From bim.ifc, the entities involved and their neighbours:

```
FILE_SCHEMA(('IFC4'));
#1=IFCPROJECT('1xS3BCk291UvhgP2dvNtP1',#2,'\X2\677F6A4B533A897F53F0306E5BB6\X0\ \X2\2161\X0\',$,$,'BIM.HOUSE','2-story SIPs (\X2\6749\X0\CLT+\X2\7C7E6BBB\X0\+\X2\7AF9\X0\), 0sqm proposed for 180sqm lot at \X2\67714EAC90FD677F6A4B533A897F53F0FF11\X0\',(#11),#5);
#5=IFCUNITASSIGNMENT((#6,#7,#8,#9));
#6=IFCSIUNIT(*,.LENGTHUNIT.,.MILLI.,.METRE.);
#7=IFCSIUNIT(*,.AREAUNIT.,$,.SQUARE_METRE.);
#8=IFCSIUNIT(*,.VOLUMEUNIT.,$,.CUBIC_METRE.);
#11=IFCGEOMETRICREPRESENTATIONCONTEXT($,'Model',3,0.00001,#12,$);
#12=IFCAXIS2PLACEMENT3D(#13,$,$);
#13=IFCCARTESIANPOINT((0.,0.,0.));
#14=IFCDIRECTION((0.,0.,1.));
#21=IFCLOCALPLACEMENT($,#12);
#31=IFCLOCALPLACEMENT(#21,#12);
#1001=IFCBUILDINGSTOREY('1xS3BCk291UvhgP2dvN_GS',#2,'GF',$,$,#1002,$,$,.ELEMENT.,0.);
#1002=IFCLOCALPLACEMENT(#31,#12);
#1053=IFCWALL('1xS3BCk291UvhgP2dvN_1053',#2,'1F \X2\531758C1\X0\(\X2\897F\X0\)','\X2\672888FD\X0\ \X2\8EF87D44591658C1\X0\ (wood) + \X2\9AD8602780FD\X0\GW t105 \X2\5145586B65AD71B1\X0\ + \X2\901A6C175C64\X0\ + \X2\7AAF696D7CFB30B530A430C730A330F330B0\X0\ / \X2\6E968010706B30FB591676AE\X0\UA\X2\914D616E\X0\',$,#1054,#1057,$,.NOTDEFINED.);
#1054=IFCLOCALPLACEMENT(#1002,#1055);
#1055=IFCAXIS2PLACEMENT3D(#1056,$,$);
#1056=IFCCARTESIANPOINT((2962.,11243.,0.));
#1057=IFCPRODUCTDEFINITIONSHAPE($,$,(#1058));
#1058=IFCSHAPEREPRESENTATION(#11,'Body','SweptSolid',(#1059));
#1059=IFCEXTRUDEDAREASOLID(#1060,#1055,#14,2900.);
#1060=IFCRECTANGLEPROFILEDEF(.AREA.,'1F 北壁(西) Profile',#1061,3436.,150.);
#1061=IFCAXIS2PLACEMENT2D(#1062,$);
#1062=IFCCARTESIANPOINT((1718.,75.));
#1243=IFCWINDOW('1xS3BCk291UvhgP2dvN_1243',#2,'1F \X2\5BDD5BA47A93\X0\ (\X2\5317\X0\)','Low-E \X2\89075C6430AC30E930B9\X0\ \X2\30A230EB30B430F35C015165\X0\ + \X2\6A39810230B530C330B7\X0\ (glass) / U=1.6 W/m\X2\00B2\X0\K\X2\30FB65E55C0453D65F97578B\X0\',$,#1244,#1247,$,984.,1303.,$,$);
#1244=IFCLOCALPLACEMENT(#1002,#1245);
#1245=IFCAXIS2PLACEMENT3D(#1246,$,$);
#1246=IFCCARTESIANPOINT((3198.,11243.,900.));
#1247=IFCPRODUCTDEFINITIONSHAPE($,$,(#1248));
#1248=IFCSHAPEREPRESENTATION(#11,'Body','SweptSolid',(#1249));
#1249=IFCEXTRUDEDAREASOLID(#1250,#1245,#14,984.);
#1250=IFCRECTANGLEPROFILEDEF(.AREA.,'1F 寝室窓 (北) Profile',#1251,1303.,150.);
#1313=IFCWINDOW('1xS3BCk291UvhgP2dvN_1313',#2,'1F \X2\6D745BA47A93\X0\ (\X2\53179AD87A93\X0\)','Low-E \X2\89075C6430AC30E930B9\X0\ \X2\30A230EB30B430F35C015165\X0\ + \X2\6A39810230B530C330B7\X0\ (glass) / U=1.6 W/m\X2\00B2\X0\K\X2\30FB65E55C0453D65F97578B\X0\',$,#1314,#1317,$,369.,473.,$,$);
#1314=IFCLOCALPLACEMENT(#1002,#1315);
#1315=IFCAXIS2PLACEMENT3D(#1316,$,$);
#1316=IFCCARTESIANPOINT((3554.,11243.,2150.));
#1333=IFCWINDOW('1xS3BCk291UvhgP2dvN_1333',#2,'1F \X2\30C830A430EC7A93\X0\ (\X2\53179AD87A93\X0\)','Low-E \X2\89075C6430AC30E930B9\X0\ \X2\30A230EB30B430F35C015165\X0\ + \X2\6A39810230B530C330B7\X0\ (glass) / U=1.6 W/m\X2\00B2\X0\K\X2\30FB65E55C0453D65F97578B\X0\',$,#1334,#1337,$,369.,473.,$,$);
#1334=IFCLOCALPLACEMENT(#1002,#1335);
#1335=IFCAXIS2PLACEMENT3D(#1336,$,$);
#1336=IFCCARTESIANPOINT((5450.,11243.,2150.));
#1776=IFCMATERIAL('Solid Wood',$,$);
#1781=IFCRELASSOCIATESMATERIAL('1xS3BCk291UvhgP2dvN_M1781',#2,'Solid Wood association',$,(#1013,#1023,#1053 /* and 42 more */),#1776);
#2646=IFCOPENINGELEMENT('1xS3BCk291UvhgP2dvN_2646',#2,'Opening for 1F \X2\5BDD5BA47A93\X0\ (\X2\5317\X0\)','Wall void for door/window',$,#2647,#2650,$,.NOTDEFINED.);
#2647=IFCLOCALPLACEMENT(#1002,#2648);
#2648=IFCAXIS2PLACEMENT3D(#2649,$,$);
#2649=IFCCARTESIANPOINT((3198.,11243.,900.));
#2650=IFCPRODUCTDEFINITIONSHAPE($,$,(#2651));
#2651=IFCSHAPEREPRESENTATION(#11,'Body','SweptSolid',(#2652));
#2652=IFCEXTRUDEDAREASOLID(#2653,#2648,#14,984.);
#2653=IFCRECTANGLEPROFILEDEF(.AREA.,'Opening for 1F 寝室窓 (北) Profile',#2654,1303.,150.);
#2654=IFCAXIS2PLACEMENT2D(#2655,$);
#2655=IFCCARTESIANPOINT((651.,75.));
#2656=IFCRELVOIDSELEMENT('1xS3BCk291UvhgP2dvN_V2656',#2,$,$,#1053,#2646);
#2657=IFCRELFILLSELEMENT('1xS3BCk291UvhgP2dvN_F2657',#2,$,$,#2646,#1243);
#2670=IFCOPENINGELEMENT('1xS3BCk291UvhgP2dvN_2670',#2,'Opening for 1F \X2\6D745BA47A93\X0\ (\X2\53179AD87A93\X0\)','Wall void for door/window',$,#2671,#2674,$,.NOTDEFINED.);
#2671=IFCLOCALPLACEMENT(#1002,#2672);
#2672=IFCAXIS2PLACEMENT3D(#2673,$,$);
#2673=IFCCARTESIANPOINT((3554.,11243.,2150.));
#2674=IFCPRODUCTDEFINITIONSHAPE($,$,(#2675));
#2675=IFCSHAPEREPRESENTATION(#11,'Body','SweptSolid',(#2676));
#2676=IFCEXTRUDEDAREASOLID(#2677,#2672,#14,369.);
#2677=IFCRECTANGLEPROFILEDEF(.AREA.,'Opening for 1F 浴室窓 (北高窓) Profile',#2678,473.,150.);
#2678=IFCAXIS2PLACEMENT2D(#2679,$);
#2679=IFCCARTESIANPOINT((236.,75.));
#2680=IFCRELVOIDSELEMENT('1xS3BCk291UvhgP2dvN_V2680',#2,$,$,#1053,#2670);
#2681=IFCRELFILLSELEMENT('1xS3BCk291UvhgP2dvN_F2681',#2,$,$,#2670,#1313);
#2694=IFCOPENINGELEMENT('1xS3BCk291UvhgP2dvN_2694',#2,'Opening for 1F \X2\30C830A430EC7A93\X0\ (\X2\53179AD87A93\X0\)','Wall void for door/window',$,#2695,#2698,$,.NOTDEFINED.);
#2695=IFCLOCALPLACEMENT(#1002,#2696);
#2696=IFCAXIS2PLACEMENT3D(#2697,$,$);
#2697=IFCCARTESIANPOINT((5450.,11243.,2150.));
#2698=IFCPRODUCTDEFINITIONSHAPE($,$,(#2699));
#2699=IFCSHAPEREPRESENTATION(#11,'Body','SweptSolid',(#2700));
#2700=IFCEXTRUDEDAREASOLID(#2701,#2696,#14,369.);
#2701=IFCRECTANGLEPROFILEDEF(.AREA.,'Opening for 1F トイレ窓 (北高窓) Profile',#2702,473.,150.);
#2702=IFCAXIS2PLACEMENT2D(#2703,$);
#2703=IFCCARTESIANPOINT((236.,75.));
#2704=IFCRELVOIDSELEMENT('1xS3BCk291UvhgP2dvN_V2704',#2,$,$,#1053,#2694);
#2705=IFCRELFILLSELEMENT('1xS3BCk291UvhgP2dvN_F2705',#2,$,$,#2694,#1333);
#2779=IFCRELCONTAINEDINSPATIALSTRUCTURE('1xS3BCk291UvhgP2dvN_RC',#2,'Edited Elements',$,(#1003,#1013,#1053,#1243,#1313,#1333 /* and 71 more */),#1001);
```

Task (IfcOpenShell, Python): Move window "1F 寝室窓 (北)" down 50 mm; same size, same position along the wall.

```python
import numpy as np
import ifcopenshell
import ifcopenshell.api.geometry
import ifcopenshell.util.placement
import ifcopenshell.util.unit

model = ifcopenshell.open("bim.ifc")
unit_scale = ifcopenshell.util.unit.calculate_unit_scale(model)

window = model.by_guid("1xS3BCk291UvhgP2dvN_1243")
opening = window.FillsVoids[0].RelatingOpeningElement
dz = -50.0

shift = np.array([0.0, 0.0, dz])
# The window is not placed relative to its opening, so move both.
for product in (opening, window):
    matrix = ifcopenshell.util.placement.get_local_placement(product.ObjectPlacement)
    matrix[:3, 3] += shift
    ifcopenshell.api.geometry.edit_object_placement(model, product=product, matrix=matrix, is_si=False)

print(f"moved by {dz * unit_scale:+.3f} m")

model.write("bim_updated.ifc")
```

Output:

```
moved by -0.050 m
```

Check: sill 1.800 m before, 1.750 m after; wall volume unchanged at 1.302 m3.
